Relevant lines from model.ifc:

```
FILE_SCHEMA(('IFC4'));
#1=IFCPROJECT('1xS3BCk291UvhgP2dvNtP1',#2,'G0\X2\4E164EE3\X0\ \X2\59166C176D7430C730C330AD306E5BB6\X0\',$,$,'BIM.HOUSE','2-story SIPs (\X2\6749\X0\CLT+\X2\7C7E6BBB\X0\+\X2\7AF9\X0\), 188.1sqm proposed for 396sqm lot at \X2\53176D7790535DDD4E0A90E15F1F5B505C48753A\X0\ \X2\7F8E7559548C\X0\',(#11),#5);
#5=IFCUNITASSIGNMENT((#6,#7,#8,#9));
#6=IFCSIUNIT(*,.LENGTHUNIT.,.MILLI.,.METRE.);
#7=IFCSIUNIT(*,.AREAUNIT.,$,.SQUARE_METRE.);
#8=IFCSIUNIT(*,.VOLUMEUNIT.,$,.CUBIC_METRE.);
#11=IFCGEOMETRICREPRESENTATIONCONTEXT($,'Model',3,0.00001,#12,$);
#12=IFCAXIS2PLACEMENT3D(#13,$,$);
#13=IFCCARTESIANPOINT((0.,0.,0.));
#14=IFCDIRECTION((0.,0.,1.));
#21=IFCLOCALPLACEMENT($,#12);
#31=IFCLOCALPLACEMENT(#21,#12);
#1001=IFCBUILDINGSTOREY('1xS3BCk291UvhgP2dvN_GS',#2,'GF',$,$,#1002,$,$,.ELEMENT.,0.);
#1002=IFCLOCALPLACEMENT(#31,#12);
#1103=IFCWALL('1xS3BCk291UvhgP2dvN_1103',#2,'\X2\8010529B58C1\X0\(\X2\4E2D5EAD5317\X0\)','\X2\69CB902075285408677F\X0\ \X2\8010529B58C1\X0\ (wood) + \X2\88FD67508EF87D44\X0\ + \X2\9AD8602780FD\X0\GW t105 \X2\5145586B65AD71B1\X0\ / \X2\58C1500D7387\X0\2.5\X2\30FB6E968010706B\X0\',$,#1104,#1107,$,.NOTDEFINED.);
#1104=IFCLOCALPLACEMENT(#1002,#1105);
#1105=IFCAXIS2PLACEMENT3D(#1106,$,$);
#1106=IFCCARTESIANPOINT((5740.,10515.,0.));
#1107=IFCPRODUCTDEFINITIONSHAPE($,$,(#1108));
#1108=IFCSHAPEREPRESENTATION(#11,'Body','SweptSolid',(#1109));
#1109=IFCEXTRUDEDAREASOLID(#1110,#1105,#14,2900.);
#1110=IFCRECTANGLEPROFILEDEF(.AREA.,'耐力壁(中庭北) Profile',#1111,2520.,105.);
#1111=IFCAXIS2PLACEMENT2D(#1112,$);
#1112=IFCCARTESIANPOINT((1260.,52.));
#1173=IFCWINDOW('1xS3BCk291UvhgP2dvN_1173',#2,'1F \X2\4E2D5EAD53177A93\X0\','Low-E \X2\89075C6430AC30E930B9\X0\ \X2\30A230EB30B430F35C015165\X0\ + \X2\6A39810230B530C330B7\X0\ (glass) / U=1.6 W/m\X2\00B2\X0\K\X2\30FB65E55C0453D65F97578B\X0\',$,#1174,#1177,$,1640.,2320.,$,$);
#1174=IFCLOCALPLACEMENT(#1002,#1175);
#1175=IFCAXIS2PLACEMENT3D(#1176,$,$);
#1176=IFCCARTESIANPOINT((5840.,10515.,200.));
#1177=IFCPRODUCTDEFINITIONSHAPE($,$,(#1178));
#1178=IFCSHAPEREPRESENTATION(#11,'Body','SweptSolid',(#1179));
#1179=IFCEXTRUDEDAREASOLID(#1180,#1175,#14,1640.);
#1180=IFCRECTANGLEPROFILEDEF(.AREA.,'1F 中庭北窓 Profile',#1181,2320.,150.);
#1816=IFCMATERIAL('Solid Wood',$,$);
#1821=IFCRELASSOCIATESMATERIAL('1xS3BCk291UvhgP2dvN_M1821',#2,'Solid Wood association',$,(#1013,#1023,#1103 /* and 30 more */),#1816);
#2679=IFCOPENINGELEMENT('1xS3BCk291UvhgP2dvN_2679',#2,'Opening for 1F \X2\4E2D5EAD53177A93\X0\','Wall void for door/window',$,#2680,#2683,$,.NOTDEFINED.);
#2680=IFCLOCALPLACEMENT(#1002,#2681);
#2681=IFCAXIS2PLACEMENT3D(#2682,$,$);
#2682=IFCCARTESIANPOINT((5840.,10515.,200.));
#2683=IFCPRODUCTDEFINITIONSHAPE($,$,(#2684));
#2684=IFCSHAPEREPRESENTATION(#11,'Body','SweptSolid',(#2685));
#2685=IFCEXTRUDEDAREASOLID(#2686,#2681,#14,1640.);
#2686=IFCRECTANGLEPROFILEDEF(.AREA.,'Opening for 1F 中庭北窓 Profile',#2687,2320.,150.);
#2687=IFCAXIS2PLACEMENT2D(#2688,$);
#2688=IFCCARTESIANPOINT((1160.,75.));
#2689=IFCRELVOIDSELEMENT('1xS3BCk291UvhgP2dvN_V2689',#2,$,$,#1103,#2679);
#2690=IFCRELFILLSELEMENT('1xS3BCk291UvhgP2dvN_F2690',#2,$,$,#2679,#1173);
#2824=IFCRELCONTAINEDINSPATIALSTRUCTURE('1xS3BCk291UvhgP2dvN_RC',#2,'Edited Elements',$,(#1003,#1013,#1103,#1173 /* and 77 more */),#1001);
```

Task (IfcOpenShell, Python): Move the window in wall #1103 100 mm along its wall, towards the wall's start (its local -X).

```python
import ifcopenshell
import ifcopenshell.api.geometry
import ifcopenshell.util.placement

model = ifcopenshell.open("model.ifc")

window = model.by_guid("1xS3BCk291UvhgP2dvN_1173")
opening = window.FillsVoids[0].RelatingOpeningElement
wall = opening.VoidsElements[0].RelatingBuildingElement

wall_matrix = ifcopenshell.util.placement.get_local_placement(wall.ObjectPlacement)
shift = wall_matrix[:3, 0] * -100.0
before = ifcopenshell.util.placement.get_local_placement(window.ObjectPlacement)[:3, 3].copy()

# The window is not placed relative to its opening, so move both.
for product in (opening, window):
    matrix = ifcopenshell.util.placement.get_local_placement(product.ObjectPlacement)
    matrix[:3, 3] += shift
    ifcopenshell.api.geometry.edit_object_placement(model, product=product, matrix=matrix, is_si=False)

after = ifcopenshell.util.placement.get_local_placement(window.ObjectPlacement)[:3, 3]
print("window moved by", (after - before).round(3) + 0.0)

model.write("model_edited.ifc")
```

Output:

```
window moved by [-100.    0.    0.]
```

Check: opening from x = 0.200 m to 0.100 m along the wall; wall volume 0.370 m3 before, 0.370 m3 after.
